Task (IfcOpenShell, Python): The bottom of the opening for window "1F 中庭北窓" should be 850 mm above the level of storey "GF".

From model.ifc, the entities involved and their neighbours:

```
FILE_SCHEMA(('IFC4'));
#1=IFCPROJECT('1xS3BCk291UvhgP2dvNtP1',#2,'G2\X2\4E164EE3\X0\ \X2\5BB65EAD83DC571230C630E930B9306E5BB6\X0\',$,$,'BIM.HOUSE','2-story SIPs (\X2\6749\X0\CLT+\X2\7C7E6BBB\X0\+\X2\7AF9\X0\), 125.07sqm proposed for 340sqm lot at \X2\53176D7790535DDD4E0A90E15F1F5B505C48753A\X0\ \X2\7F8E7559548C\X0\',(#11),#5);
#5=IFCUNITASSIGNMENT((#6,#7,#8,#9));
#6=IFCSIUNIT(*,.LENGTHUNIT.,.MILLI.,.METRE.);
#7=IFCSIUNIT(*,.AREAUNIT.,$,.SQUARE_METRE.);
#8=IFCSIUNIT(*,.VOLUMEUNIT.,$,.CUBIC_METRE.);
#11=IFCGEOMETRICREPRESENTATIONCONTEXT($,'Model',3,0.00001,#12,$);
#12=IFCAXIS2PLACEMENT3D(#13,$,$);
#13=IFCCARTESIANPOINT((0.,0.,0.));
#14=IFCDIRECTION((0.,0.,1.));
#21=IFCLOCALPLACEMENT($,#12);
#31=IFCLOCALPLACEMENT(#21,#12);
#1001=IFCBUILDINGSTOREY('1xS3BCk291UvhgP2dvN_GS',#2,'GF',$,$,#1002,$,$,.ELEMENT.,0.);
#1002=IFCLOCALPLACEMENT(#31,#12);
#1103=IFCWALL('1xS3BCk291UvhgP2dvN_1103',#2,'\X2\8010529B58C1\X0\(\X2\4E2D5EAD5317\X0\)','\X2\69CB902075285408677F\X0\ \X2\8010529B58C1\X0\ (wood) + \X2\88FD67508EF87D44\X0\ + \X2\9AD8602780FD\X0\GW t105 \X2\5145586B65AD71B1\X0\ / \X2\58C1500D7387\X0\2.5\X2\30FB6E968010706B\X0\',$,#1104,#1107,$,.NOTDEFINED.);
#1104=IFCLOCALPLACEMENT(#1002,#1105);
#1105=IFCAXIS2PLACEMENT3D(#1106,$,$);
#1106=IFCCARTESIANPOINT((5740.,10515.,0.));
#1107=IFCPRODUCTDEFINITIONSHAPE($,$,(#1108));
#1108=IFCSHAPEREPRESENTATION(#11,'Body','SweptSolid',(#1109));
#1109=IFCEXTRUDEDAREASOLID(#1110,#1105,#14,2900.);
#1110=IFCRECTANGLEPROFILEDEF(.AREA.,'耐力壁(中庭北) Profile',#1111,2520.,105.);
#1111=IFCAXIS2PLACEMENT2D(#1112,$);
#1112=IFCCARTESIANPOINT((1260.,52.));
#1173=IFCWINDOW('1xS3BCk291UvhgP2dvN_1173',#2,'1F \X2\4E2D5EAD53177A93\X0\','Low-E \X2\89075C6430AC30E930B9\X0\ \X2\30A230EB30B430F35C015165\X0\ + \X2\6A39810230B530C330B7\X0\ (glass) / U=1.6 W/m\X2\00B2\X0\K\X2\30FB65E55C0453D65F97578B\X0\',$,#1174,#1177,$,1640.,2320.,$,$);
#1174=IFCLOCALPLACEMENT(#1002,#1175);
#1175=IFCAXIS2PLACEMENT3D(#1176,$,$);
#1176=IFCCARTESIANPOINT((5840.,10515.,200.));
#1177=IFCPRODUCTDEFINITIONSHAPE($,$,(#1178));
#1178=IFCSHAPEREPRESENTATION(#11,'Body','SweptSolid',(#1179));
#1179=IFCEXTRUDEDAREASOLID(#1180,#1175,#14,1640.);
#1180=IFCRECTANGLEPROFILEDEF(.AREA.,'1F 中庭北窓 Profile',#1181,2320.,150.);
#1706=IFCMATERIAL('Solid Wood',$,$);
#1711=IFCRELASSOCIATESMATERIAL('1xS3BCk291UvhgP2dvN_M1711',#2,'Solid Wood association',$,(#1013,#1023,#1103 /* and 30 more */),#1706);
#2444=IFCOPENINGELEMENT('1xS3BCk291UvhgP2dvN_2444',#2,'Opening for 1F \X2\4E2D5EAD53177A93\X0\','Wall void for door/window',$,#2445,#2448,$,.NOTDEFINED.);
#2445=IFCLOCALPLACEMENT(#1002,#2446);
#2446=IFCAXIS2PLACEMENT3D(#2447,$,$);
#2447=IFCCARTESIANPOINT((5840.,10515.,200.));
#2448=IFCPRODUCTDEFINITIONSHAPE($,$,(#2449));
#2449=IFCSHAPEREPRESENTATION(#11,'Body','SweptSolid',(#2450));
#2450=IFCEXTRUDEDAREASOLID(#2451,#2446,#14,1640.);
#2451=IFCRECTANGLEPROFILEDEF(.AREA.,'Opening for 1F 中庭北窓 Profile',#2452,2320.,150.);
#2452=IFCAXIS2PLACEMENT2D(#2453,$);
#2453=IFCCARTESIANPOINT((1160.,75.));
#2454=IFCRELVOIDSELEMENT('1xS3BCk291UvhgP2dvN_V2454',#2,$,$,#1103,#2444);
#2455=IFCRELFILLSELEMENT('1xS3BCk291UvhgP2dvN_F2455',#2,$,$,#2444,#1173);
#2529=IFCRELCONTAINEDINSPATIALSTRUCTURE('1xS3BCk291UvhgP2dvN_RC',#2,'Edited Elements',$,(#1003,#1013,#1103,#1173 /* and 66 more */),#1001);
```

```python
import numpy as np
import ifcopenshell
import ifcopenshell.api.geometry
import ifcopenshell.geom
import ifcopenshell.util.element
import ifcopenshell.util.placement
import ifcopenshell.util.shape
import ifcopenshell.util.unit

model = ifcopenshell.open("model.ifc")
unit_scale = ifcopenshell.util.unit.calculate_unit_scale(model)

window = model.by_id(1173)
opening = window.FillsVoids[0].RelatingOpeningElement
storey = ifcopenshell.util.element.get_container(window, ifc_class="IfcBuildingStorey")
level = ifcopenshell.util.placement.get_local_placement(storey.ObjectPlacement)[2, 3]

# The opening's origin need not be at the sill, so measure its lowest point.
shape = ifcopenshell.geom.create_shape(ifcopenshell.geom.settings(), opening)
bottom = ifcopenshell.util.shape.get_shape_bottom_elevation(shape, shape.geometry) / unit_scale
dz = level + 0.85 / unit_scale - bottom

shift = np.array([0.0, 0.0, dz])
# The window is not placed relative to its opening, so move both.
for product in (opening, window):
    matrix = ifcopenshell.util.placement.get_local_placement(product.ObjectPlacement)
    matrix[:3, 3] += shift
    ifcopenshell.api.geometry.edit_object_placement(model, product=product, matrix=matrix, is_si=False)

print(f"moved by {dz * unit_scale:+.3f} m")

model.write("model_v2.ifc")
```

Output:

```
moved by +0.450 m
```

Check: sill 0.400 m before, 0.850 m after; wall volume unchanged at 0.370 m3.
